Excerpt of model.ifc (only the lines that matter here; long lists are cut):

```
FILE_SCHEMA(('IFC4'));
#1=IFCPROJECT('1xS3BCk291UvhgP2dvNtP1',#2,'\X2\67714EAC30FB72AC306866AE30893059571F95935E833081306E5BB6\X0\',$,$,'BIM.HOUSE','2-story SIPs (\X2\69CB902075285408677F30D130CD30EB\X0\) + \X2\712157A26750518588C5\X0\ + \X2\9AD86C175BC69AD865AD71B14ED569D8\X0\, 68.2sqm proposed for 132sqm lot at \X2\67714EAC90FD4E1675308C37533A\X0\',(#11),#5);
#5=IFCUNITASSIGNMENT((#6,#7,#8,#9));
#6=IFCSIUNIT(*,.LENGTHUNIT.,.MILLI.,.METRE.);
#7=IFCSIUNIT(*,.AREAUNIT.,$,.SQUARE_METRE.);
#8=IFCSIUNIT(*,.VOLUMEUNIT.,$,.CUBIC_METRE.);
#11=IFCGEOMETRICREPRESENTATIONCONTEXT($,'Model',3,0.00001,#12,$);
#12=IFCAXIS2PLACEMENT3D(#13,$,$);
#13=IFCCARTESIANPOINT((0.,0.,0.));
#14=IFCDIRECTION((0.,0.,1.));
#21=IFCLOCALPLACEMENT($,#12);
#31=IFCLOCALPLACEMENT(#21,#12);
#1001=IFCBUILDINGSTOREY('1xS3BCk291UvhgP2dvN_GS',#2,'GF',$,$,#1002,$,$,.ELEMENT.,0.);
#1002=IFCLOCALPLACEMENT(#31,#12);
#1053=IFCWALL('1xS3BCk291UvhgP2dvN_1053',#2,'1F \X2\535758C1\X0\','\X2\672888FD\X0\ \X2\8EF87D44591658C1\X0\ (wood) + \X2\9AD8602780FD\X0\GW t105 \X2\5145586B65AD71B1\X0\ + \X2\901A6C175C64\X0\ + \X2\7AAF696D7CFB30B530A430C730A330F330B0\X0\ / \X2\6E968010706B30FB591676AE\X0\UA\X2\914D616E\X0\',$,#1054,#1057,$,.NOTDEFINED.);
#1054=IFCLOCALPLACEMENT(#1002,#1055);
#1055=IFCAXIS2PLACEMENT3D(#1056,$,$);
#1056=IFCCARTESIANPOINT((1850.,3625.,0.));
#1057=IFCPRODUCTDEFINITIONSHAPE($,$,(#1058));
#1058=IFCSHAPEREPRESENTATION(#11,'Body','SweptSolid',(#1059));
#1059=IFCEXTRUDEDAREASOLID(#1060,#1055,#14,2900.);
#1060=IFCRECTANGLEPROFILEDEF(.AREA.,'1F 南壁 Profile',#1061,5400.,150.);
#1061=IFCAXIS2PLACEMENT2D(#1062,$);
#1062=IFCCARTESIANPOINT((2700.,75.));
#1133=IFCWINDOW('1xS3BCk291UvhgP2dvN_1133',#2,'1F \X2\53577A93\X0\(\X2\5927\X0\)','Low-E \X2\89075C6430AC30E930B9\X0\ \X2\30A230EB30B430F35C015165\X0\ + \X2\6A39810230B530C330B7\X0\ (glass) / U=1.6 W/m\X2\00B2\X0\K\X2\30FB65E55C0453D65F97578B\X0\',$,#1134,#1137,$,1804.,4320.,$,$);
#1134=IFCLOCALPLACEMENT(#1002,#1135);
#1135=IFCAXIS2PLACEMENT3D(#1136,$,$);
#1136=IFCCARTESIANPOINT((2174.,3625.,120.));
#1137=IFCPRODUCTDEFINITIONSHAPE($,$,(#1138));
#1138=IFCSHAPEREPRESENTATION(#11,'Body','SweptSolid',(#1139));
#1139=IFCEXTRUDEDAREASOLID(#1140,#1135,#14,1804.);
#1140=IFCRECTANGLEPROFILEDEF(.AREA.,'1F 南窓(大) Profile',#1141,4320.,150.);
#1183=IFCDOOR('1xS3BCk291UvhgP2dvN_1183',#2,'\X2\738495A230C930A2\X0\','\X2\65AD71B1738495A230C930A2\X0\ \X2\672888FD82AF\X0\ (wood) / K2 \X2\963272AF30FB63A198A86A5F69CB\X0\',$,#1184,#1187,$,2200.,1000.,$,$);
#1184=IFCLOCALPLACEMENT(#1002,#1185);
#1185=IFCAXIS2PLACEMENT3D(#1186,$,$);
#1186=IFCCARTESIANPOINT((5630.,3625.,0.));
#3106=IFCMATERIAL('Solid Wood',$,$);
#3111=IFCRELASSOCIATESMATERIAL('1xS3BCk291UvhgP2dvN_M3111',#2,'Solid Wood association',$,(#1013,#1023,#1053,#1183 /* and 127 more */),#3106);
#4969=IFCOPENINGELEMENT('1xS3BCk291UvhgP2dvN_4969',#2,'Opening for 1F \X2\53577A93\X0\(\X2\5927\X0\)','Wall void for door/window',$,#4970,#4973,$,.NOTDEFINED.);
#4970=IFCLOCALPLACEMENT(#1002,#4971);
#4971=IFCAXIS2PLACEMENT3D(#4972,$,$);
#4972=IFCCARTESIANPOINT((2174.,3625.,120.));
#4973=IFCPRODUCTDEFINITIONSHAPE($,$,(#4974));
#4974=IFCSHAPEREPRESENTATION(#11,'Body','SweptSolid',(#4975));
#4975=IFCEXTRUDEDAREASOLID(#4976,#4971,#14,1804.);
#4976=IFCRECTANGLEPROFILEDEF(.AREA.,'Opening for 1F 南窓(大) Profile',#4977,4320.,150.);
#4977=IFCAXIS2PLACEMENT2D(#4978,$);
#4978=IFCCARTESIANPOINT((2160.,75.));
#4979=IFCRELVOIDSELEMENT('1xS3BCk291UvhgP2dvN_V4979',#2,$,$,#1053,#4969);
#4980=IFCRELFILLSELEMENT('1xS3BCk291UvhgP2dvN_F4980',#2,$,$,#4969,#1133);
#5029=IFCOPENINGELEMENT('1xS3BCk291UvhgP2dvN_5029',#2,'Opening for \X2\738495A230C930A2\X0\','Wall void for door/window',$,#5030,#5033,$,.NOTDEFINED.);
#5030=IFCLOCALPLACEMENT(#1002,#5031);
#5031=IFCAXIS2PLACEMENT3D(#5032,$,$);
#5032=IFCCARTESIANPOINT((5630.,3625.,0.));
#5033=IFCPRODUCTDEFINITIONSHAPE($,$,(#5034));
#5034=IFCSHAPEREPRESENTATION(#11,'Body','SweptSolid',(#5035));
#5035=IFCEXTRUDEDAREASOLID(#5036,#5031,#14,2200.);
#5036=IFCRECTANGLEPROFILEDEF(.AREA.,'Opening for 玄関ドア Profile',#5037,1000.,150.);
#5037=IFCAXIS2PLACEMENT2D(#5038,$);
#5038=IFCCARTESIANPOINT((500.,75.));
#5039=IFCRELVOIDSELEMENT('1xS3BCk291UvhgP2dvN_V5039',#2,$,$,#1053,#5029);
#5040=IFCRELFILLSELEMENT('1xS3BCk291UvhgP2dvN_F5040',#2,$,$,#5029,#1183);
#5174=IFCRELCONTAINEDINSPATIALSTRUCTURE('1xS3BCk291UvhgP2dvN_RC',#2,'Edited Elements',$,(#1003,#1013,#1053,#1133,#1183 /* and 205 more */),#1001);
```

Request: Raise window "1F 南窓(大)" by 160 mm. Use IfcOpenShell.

```python
import numpy as np
import ifcopenshell
import ifcopenshell.api.geometry
import ifcopenshell.util.placement
import ifcopenshell.util.unit

model = ifcopenshell.open("model.ifc")
unit_scale = ifcopenshell.util.unit.calculate_unit_scale(model)

window = model.by_guid("1xS3BCk291UvhgP2dvN_1133")
opening = window.FillsVoids[0].RelatingOpeningElement
dz = 160.0

shift = np.array([0.0, 0.0, dz])
# The window is not placed relative to its opening, so move both.
for product in (opening, window):
    matrix = ifcopenshell.util.placement.get_local_placement(product.ObjectPlacement)
    matrix[:3, 3] += shift
    ifcopenshell.api.geometry.edit_object_placement(model, product=product, matrix=matrix, is_si=False)

print(f"moved by {dz * unit_scale:+.3f} m")

model.write("model_rev.ifc")
```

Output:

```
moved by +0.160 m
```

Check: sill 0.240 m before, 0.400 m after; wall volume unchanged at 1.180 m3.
